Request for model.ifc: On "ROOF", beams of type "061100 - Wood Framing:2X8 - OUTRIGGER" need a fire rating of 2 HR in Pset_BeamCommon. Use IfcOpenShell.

First a look at what the model holds.

```python
import ifcopenshell
import ifcopenshell.util.element

model = ifcopenshell.open("model.ifc")
print(model.schema)
storey = next(s for s in model.by_type("IfcBuildingStorey") if s.Name == "ROOF")
beams = [e for e in ifcopenshell.util.element.get_decomposition(storey) if e.is_a("IfcBeam")]
seen = {}
for e in beams:
    element_type = ifcopenshell.util.element.get_type(e)
    key = (element_type.Name if element_type != e and element_type else None, ifcopenshell.util.element.get_pset(e, "Pset_BeamCommon", "FireRating"))
    seen[key] = seen.get(key, 0) + 1
for (name, value), count in sorted(seen.items(), key=str):
    print(count, "x", name, "|", value)
```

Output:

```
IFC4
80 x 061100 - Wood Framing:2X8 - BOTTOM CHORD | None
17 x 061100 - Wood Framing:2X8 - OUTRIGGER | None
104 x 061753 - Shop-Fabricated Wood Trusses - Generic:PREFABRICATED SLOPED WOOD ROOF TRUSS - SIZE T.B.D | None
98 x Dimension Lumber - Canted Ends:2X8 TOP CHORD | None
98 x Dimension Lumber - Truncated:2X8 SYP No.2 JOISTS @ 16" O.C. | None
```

```python
import ifcopenshell
import ifcopenshell.api.pset
import ifcopenshell.util.element

model = ifcopenshell.open("model.ifc")

storey = next(s for s in model.by_type("IfcBuildingStorey") if s.Name == "ROOF")
beams = [e for e in ifcopenshell.util.element.get_decomposition(storey) if e.is_a("IfcBeam")]

count = 0
for e in beams:
    element_type = ifcopenshell.util.element.get_type(e)
    if element_type in (None, e) or element_type.Name != "061100 - Wood Framing:2X8 - OUTRIGGER":
        continue
    # add_pset returns the element's existing set when there is one.
    pset = ifcopenshell.api.pset.add_pset(model, product=e, name="Pset_BeamCommon")
    ifcopenshell.api.pset.edit_pset(model, pset=pset, properties={"FireRating": "2 HR"})
    count += 1

print(count, "beams updated")

model.write("model_updated.ifc")
```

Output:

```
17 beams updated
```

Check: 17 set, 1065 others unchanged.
